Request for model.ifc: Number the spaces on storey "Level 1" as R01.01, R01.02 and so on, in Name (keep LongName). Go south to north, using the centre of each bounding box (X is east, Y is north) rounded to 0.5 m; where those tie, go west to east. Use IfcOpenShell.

First a look at what the model holds.

```python
import ifcopenshell
import ifcopenshell.util.element
import ifcopenshell.util.placement

model = ifcopenshell.open("model.ifc")
print(model.schema)
storey = next(s for s in model.by_type("IfcBuildingStorey") if s.Name == "Level 1")
spaces = [e for e in ifcopenshell.util.element.get_decomposition(storey) if e.is_a("IfcSpace")]
for e in sorted(spaces, key=lambda e: e.id()):
    origin = ifcopenshell.util.placement.get_local_placement(e.ObjectPlacement)[:3, 3]
    print(e.id(), e.Name, e.LongName, origin.round(2) + 0.0, sep=" | ")
```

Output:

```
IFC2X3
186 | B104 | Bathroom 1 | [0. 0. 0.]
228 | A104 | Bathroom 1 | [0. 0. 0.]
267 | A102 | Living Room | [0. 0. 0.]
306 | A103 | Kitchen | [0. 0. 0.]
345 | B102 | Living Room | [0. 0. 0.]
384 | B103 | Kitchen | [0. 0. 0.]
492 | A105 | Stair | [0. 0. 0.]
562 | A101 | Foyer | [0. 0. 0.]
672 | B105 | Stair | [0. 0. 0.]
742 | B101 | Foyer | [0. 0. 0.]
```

```python
import ifcopenshell
import ifcopenshell.geom
import ifcopenshell.util.element
import ifcopenshell.util.shape

model = ifcopenshell.open("model.ifc")
settings = ifcopenshell.geom.settings()
settings.set("use-world-coords", True)


def centre(element):
    shape = ifcopenshell.geom.create_shape(settings, element)
    return ifcopenshell.util.shape.get_bbox_centroid(shape.geometry)


storey = next(s for s in model.by_type("IfcBuildingStorey") if s.Name == "Level 1")
spaces = [e for e in ifcopenshell.util.element.get_decomposition(storey) if e.is_a("IfcSpace")]

# Insertion points can sit at a corner or the storey origin, so sort by the geometry (in metres).
centres = {e: centre(e) for e in spaces}
spaces.sort(key=lambda e: (round(centres[e][1] / 0.5), centres[e][0]))

for i, e in enumerate(spaces, start=1):
    number = f"R01.{i:02d}"
    e.Name = number
    print(e.id(), number)

model.write("model_edited.ifc")
```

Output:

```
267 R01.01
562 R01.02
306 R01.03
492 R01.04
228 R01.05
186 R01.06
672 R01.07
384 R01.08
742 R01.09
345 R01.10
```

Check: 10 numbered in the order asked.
